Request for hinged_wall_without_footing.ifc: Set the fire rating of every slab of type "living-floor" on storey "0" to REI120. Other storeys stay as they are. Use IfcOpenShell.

First a look at what the model holds.

```python
import ifcopenshell
import ifcopenshell.util.element

model = ifcopenshell.open("hinged_wall_without_footing.ifc")
print(model.schema)
storey = next(s for s in model.by_type("IfcBuildingStorey") if s.Name == "0")
slabs = [e for e in ifcopenshell.util.element.get_decomposition(storey) if e.is_a("IfcSlab")]
seen = {}
for e in slabs:
    element_type = ifcopenshell.util.element.get_type(e)
    key = (element_type.Name if element_type != e and element_type else None, ifcopenshell.util.element.get_pset(e, "Pset_SlabCommon", "FireRating"))
    seen[key] = seen.get(key, 0) + 1
for (name, value), count in sorted(seen.items(), key=str):
    print(count, "x", name, "|", value)
```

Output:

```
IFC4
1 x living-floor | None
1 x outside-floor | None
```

```python
import ifcopenshell
import ifcopenshell.api.pset
import ifcopenshell.util.element

model = ifcopenshell.open("hinged_wall_without_footing.ifc")

storey = next(s for s in model.by_type("IfcBuildingStorey") if s.Name == "0")
slabs = [e for e in ifcopenshell.util.element.get_decomposition(storey) if e.is_a("IfcSlab")]

count = 0
for e in slabs:
    element_type = ifcopenshell.util.element.get_type(e)
    if element_type in (None, e) or element_type.Name != "living-floor":
        continue
    # add_pset returns the element's existing set when there is one.
    pset = ifcopenshell.api.pset.add_pset(model, product=e, name="Pset_SlabCommon")
    ifcopenshell.api.pset.edit_pset(model, pset=pset, properties={"FireRating": "REI120"})
    count += 1

print(count, "slabs updated")

model.write("hinged_wall_without_footing_updated.ifc")
```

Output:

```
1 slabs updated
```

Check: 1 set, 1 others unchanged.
